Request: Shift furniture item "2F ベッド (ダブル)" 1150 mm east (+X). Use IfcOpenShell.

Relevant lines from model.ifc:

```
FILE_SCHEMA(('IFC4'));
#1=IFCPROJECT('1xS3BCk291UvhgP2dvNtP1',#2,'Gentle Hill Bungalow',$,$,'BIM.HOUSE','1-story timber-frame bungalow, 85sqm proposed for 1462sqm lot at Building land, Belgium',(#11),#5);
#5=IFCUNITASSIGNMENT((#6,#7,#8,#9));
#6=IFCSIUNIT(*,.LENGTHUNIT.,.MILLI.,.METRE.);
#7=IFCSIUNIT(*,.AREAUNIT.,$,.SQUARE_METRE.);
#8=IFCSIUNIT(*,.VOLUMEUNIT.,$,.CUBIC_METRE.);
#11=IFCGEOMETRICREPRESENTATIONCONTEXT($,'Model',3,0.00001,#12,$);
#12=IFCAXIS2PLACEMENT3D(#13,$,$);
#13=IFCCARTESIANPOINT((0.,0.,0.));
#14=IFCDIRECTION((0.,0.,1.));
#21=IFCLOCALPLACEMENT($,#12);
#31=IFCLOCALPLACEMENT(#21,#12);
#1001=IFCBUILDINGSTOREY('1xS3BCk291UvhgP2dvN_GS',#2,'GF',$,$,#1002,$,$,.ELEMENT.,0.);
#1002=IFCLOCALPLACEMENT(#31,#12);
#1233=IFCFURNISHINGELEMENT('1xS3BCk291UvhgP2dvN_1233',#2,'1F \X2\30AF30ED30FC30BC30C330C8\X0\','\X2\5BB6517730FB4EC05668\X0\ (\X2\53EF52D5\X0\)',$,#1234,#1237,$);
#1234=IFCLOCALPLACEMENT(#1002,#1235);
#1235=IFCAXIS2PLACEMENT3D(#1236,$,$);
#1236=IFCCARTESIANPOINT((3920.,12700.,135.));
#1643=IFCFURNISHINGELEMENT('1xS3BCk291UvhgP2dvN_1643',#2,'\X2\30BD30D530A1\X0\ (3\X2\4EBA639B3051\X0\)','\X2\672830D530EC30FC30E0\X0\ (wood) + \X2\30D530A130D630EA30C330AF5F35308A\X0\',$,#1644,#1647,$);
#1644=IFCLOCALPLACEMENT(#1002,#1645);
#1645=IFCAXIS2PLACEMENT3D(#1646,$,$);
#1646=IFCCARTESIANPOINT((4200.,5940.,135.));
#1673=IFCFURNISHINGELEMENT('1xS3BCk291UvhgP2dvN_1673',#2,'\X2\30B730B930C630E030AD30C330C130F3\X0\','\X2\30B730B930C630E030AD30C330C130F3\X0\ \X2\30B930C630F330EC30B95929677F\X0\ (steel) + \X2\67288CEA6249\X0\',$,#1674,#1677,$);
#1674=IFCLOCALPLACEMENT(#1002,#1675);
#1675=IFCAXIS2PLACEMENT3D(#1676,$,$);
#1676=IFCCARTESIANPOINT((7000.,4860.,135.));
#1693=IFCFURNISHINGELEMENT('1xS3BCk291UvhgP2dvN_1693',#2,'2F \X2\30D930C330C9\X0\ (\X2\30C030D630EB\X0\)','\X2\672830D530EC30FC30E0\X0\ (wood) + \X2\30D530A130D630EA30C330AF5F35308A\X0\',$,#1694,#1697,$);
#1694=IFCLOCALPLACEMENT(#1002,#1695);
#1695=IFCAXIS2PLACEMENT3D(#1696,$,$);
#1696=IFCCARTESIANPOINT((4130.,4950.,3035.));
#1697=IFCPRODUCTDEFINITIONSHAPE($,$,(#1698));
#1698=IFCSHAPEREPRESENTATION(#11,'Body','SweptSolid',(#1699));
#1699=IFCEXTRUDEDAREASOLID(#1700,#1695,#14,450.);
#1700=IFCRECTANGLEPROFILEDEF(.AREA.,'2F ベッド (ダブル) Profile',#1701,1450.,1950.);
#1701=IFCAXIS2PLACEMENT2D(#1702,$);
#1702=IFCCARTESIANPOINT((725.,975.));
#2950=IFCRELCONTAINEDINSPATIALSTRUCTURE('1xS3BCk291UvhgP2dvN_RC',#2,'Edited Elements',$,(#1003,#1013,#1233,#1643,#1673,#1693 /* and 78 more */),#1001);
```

```python
import ifcopenshell
import ifcopenshell.api.geometry
import ifcopenshell.util.placement
import ifcopenshell.util.unit

model = ifcopenshell.open("model.ifc")
unit_scale = ifcopenshell.util.unit.calculate_unit_scale(model)

item = model.by_id(1693)
matrix = ifcopenshell.util.placement.get_local_placement(item.ObjectPlacement)
matrix[0, 3] += 1.15 / unit_scale
ifcopenshell.api.geometry.edit_object_placement(model, product=item, matrix=matrix, is_si=False)

print(ifcopenshell.util.placement.get_local_placement(item.ObjectPlacement).round(3) + 0.0)

model.write("model-out.ifc")
```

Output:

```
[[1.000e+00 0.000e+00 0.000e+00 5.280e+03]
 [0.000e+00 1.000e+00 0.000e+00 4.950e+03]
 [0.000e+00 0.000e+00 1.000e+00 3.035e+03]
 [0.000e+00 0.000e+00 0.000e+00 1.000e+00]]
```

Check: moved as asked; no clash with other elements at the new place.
